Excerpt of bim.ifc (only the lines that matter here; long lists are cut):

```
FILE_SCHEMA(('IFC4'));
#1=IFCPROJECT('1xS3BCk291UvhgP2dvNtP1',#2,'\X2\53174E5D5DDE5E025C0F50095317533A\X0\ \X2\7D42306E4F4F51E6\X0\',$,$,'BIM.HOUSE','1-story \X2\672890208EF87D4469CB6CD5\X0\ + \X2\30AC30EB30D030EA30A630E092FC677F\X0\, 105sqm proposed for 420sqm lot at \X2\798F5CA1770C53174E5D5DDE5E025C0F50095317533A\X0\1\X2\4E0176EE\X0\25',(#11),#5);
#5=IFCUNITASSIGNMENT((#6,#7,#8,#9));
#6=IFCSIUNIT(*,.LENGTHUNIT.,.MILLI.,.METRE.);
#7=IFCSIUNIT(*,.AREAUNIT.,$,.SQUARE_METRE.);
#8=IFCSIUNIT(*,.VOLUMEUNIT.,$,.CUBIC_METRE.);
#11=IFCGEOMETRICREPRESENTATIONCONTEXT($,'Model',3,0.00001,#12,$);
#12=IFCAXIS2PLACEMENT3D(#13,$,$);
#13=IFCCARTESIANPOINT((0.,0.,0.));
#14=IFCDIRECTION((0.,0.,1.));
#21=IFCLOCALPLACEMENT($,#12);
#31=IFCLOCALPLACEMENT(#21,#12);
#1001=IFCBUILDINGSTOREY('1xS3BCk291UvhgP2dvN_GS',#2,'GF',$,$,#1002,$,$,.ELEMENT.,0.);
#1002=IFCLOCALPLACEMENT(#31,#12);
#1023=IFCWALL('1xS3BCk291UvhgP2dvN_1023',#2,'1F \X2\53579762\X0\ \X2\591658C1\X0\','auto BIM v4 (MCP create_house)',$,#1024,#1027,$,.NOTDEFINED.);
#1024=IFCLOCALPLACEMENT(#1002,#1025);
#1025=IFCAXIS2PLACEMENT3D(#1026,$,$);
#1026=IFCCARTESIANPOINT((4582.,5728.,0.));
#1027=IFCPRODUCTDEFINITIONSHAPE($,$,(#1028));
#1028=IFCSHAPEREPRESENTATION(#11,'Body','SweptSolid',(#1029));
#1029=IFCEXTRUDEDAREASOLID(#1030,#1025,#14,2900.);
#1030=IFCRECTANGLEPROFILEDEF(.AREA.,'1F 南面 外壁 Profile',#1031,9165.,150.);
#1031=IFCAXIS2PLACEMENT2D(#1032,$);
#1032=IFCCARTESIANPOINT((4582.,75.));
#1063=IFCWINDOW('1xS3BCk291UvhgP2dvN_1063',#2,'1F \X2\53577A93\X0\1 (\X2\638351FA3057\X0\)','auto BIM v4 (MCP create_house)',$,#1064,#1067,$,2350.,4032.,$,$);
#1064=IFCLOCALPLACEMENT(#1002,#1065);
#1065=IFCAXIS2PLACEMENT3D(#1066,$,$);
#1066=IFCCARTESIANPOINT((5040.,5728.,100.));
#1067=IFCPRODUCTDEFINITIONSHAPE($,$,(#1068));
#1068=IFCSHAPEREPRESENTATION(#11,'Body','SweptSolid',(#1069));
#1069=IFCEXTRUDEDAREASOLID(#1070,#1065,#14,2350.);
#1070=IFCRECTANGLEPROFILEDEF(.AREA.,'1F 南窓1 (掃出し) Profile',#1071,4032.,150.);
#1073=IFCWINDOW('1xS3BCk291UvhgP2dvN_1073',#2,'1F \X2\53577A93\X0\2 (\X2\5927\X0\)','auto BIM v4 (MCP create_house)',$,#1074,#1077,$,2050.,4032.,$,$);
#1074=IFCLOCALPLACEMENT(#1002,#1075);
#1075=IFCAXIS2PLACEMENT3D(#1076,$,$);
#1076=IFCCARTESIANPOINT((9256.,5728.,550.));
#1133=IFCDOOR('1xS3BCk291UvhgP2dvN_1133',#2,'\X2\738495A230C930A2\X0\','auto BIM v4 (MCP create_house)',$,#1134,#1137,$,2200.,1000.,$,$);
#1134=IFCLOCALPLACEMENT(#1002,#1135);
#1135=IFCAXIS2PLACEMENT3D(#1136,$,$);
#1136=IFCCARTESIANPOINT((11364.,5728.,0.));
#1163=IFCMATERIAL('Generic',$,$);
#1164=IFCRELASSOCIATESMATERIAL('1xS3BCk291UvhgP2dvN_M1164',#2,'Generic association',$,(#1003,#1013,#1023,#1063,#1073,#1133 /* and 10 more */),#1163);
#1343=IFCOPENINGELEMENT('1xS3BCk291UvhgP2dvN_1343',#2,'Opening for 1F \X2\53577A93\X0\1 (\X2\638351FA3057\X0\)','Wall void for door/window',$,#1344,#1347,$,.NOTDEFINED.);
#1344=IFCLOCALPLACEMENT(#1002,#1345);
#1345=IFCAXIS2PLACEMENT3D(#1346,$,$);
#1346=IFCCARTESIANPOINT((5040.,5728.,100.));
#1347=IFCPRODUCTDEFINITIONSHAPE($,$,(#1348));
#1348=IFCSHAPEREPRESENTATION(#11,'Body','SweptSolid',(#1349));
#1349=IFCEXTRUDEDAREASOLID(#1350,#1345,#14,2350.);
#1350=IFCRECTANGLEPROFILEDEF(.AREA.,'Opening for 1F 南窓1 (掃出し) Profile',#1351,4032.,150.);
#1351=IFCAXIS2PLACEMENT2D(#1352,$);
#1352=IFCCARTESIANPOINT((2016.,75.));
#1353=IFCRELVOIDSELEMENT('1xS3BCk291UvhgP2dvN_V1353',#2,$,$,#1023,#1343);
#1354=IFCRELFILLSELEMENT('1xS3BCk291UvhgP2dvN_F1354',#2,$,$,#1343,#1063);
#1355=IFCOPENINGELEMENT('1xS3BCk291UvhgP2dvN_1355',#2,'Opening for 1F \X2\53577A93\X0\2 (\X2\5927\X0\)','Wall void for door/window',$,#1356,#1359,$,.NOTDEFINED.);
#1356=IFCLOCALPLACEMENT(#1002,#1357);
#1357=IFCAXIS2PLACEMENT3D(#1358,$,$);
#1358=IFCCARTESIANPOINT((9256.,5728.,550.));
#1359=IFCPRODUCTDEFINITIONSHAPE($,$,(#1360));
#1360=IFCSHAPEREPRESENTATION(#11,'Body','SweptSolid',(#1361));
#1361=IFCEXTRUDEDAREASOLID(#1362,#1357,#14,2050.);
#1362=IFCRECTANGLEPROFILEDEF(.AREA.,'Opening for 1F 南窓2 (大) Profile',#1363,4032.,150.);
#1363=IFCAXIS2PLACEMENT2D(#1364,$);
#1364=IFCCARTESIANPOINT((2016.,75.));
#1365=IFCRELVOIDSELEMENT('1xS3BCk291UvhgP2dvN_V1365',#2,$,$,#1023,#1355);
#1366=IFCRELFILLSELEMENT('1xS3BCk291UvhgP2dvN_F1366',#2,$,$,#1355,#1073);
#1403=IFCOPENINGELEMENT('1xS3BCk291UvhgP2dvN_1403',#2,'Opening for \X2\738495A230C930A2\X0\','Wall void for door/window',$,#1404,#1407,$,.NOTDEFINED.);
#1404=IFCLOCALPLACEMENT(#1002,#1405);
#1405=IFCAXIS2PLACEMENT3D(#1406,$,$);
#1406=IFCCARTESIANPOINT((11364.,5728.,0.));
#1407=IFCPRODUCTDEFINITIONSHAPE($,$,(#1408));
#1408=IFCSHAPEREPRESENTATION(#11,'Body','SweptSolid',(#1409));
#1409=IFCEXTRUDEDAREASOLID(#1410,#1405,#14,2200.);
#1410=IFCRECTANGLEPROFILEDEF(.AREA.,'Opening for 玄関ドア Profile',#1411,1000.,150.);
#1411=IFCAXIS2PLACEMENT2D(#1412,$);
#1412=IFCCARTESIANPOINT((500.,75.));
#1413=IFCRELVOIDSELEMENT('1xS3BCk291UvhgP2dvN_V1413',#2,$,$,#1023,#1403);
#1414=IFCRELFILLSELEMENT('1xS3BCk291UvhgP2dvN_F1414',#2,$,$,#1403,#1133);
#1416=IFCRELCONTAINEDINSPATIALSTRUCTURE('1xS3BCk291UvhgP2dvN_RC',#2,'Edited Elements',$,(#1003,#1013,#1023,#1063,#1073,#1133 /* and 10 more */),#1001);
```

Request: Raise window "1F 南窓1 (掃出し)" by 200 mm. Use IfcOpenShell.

```python
import numpy as np
import ifcopenshell
import ifcopenshell.api.geometry
import ifcopenshell.util.placement
import ifcopenshell.util.unit

model = ifcopenshell.open("bim.ifc")
unit_scale = ifcopenshell.util.unit.calculate_unit_scale(model)

window = model.by_guid("1xS3BCk291UvhgP2dvN_1063")
opening = window.FillsVoids[0].RelatingOpeningElement
dz = 0.2 / unit_scale

shift = np.array([0.0, 0.0, dz])
# The window is not placed relative to its opening, so move both.
for product in (opening, window):
    matrix = ifcopenshell.util.placement.get_local_placement(product.ObjectPlacement)
    matrix[:3, 3] += shift
    ifcopenshell.api.geometry.edit_object_placement(model, product=product, matrix=matrix, is_si=False)

print(f"moved by {dz * unit_scale:+.3f} m")

model.write("bim_updated.ifc")
```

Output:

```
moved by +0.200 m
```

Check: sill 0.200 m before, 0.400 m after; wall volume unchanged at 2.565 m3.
